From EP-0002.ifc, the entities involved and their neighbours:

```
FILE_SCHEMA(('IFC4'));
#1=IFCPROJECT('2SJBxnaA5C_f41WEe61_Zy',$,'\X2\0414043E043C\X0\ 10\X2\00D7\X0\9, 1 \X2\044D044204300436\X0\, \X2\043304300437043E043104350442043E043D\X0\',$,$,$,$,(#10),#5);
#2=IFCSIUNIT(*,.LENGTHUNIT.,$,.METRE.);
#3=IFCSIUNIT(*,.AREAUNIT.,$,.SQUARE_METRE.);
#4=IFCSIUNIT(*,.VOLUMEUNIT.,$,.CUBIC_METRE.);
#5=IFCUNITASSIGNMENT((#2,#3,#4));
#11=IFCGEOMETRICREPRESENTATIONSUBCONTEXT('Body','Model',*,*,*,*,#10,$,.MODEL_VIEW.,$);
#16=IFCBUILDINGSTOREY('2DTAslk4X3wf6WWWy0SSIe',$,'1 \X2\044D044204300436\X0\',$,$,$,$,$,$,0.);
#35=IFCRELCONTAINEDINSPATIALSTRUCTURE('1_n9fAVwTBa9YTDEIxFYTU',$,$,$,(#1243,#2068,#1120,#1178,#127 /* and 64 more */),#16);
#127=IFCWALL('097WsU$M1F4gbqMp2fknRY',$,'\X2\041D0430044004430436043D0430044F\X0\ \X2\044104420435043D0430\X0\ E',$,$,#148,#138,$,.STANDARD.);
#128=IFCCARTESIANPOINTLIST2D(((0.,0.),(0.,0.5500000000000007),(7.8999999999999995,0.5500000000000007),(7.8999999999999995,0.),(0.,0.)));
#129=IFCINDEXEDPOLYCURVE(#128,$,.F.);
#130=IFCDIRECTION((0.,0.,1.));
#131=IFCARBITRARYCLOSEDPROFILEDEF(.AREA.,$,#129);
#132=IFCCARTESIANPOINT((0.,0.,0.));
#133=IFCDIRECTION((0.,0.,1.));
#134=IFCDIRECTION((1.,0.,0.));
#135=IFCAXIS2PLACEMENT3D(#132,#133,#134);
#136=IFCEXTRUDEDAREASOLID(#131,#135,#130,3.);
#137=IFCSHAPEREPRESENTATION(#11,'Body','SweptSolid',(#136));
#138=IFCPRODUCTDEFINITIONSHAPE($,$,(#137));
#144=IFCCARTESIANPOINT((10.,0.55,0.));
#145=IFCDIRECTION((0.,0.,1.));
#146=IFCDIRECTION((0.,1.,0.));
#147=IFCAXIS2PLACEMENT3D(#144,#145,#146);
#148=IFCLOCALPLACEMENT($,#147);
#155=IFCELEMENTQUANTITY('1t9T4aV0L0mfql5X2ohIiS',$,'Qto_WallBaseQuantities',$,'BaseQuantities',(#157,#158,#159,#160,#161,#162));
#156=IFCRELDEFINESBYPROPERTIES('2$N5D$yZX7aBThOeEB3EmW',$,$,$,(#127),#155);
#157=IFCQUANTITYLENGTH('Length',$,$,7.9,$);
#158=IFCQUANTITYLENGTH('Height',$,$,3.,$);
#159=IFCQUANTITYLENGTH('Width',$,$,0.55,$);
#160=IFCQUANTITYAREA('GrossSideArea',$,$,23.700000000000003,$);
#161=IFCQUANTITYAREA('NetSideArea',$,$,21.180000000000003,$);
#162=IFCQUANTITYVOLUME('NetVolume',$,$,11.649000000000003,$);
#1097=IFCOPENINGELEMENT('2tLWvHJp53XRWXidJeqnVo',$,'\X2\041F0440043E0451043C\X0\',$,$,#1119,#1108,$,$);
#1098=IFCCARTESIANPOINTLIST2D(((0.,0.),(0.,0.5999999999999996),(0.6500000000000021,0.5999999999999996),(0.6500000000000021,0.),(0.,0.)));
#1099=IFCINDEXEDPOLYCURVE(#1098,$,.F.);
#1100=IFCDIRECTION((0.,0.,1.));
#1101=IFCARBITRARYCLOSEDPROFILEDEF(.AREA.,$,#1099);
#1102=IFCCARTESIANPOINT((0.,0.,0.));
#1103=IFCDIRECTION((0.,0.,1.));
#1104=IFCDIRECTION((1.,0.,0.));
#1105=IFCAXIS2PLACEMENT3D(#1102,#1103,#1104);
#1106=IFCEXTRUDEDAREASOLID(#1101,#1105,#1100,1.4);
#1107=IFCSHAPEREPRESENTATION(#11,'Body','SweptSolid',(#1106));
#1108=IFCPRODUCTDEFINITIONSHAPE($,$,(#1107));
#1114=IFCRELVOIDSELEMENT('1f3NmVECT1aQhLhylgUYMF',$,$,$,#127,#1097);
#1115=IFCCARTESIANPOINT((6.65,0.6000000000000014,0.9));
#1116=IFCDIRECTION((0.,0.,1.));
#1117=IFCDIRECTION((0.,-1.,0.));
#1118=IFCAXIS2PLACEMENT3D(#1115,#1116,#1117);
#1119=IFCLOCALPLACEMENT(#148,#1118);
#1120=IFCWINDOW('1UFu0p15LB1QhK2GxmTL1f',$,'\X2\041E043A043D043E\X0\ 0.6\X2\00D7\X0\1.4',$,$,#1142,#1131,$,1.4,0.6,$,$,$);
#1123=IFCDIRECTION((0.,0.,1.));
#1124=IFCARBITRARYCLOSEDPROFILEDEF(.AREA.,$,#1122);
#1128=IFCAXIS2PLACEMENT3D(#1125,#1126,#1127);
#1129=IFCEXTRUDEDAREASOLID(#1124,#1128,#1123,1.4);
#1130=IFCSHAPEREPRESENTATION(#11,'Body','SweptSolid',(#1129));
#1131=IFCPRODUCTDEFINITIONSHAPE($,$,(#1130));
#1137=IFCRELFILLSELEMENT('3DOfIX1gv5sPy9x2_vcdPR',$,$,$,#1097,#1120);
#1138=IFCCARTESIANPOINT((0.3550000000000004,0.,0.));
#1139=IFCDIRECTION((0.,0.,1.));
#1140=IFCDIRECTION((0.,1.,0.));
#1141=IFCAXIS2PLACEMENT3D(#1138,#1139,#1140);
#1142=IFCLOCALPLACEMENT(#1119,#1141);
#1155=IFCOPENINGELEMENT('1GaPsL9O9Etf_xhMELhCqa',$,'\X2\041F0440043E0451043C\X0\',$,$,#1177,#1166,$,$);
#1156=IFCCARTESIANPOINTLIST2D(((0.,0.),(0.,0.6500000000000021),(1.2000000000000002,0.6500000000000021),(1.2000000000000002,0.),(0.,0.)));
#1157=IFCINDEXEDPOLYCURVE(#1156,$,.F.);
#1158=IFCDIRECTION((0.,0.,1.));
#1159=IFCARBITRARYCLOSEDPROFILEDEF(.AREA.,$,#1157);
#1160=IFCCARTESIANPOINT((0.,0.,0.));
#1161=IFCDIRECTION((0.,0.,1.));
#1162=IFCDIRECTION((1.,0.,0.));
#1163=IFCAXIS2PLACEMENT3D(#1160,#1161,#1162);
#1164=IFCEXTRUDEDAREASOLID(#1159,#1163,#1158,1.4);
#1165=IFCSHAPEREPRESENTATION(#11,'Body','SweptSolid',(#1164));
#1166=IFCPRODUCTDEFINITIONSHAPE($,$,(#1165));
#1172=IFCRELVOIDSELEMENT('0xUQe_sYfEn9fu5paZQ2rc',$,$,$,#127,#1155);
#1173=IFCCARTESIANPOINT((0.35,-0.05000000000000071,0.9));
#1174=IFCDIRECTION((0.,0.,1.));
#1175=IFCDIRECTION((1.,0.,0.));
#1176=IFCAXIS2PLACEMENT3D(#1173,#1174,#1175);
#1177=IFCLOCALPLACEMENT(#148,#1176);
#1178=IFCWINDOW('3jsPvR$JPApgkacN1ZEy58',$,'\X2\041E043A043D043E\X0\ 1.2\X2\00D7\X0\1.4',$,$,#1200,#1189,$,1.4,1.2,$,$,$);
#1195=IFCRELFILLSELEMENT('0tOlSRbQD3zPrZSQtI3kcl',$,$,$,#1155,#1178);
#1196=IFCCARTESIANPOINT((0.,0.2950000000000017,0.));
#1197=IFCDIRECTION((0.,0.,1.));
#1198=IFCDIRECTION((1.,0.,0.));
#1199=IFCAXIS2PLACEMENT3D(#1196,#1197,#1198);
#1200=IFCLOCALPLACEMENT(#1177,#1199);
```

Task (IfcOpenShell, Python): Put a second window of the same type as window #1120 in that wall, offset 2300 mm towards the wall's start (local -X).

```python
import ifcopenshell
import ifcopenshell.api.feature
import ifcopenshell.api.geometry
import ifcopenshell.api.pset
import ifcopenshell.api.root
import ifcopenshell.geom
import ifcopenshell.util.element
import ifcopenshell.util.placement
import ifcopenshell.util.shape
import ifcopenshell.util.unit

model = ifcopenshell.open("EP-0002.ifc")
unit_scale = ifcopenshell.util.unit.calculate_unit_scale(model)
area_scale = ifcopenshell.util.unit.calculate_unit_scale(model, "AREAUNIT")
volume_scale = ifcopenshell.util.unit.calculate_unit_scale(model, "VOLUMEUNIT")
settings = ifcopenshell.geom.settings()


def volume(element):
    """Net volume in cubic metres, openings subtracted."""
    shape = ifcopenshell.geom.create_shape(settings, element)
    return ifcopenshell.util.shape.get_volume(shape.geometry)


window = model.by_guid("1UFu0p15LB1QhK2GxmTL1f")
opening = window.FillsVoids[0].RelatingOpeningElement
wall = opening.VoidsElements[0].RelatingBuildingElement
before = volume(wall)
shift = ifcopenshell.util.placement.get_local_placement(wall.ObjectPlacement)[:3, 0] * -2.3 / unit_scale

# copy_class copies the void relationship, type, container and properties, but no geometry.
new_opening = ifcopenshell.api.root.copy_class(model, product=opening)
new_opening.Representation = ifcopenshell.util.element.copy_deep(
    model, opening.Representation, exclude=["IfcGeometricRepresentationContext", "IfcRepresentationMap"]
)
new_window = ifcopenshell.api.root.copy_class(model, product=window)
new_window.Representation = ifcopenshell.util.element.copy_deep(
    model, window.Representation, exclude=["IfcGeometricRepresentationContext", "IfcRepresentationMap"]
)
ifcopenshell.api.feature.add_filling(model, opening=new_opening, element=new_window)

for old, new in ((opening, new_opening), (window, new_window)):
    matrix = ifcopenshell.util.placement.get_local_placement(old.ObjectPlacement)
    matrix[:3, 3] += shift
    ifcopenshell.api.geometry.edit_object_placement(model, product=new, matrix=matrix, is_si=False)

after = volume(wall)
thickness = 0.55  # wall thickness in metres

# Update the wall's stored quantities.
qto = model.by_id(ifcopenshell.util.element.get_pset(wall, "Qto_WallBaseQuantities", should_inherit=False)["id"])
ifcopenshell.api.pset.edit_qto(model, qto=qto, properties={
    "NetSideArea": after / thickness / area_scale,
    "NetVolume": after / volume_scale,
})

print(f"wall volume {before:.3f} -> {after:.3f} m3")

model.write("EP-0002_updated.ifc")
```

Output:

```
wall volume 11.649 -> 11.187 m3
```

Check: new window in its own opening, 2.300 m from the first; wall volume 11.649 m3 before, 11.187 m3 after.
